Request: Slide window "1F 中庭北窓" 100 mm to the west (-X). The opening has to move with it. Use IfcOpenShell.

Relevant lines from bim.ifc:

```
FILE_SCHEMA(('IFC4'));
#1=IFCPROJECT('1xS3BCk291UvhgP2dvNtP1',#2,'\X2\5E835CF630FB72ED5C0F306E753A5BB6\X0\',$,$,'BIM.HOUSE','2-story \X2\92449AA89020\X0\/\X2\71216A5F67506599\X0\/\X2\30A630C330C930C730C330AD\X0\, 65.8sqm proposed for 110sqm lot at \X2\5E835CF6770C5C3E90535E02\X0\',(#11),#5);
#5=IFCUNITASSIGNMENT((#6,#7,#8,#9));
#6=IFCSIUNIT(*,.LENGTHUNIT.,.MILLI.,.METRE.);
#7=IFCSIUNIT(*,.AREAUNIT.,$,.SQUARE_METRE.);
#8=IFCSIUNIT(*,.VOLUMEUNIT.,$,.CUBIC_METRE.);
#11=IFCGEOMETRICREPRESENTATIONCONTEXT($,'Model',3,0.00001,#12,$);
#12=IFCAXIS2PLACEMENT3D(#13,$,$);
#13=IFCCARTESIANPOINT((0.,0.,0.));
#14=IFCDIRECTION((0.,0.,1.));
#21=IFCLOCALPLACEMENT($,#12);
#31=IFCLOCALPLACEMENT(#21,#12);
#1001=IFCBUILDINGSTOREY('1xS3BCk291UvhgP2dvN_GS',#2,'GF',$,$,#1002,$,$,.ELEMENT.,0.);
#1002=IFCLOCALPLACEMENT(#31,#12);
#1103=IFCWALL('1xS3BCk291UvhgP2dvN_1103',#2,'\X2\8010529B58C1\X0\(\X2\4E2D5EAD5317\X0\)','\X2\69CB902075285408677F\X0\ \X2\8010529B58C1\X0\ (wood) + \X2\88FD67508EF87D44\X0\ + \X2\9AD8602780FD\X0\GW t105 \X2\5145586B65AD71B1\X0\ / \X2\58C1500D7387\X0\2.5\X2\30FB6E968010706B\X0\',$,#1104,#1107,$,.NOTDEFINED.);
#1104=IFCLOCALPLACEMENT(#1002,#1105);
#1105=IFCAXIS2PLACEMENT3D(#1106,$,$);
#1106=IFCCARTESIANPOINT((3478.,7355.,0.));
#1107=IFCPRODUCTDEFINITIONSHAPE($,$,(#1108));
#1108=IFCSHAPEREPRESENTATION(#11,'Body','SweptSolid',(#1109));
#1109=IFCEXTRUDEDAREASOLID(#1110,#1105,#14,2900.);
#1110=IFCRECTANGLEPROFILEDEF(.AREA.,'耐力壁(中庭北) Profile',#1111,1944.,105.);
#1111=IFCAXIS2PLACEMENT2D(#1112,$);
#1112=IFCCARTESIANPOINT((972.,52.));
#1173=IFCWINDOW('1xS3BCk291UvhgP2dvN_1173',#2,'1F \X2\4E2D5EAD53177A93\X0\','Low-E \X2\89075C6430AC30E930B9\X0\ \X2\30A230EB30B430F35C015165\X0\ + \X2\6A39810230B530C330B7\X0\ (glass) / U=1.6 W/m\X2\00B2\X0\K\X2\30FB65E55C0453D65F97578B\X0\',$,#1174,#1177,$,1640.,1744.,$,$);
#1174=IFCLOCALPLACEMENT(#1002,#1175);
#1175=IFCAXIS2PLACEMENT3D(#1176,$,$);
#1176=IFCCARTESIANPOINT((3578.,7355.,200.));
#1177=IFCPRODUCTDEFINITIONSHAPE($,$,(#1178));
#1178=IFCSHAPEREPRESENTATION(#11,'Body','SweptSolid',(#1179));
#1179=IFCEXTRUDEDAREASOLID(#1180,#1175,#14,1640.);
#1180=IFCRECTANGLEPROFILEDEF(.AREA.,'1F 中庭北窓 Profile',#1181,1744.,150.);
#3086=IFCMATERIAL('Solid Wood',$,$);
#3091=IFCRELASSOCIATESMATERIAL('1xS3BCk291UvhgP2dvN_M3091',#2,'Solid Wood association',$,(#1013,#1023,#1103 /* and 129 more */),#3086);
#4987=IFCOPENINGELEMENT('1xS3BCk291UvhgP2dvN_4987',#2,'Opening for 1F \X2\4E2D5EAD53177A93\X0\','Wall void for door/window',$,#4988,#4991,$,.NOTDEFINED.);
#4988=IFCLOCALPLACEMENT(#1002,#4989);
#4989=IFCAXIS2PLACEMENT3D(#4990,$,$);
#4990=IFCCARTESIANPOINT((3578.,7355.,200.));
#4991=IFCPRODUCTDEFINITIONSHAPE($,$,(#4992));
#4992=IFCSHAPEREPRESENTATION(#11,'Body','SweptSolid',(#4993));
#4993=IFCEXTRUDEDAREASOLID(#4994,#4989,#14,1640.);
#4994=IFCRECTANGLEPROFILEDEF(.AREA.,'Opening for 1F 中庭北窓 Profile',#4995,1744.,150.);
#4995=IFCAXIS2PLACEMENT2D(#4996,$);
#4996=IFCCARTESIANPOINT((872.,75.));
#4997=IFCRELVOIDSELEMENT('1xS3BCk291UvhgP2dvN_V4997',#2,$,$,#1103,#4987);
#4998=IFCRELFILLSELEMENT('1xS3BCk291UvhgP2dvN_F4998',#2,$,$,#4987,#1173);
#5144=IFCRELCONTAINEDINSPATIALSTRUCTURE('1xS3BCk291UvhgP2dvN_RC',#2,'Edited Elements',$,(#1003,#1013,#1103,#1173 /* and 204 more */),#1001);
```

```python
import ifcopenshell
import ifcopenshell.api.geometry
import ifcopenshell.util.placement
import ifcopenshell.util.unit

model = ifcopenshell.open("bim.ifc")
unit_scale = ifcopenshell.util.unit.calculate_unit_scale(model)

window = model.by_id(1173)
opening = window.FillsVoids[0].RelatingOpeningElement
wall = opening.VoidsElements[0].RelatingBuildingElement

wall_matrix = ifcopenshell.util.placement.get_local_placement(wall.ObjectPlacement)
shift = wall_matrix[:3, 0] * -0.1 / unit_scale
before = ifcopenshell.util.placement.get_local_placement(window.ObjectPlacement)[:3, 3].copy()

# The window is not placed relative to its opening, so move both.
for product in (opening, window):
    matrix = ifcopenshell.util.placement.get_local_placement(product.ObjectPlacement)
    matrix[:3, 3] += shift
    ifcopenshell.api.geometry.edit_object_placement(model, product=product, matrix=matrix, is_si=False)

after = ifcopenshell.util.placement.get_local_placement(window.ObjectPlacement)[:3, 3]
print("window moved by", (after - before).round(3) + 0.0)

model.write("bim-out.ifc")
```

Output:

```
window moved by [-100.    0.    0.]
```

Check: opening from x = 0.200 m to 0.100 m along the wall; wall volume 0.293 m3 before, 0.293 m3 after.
